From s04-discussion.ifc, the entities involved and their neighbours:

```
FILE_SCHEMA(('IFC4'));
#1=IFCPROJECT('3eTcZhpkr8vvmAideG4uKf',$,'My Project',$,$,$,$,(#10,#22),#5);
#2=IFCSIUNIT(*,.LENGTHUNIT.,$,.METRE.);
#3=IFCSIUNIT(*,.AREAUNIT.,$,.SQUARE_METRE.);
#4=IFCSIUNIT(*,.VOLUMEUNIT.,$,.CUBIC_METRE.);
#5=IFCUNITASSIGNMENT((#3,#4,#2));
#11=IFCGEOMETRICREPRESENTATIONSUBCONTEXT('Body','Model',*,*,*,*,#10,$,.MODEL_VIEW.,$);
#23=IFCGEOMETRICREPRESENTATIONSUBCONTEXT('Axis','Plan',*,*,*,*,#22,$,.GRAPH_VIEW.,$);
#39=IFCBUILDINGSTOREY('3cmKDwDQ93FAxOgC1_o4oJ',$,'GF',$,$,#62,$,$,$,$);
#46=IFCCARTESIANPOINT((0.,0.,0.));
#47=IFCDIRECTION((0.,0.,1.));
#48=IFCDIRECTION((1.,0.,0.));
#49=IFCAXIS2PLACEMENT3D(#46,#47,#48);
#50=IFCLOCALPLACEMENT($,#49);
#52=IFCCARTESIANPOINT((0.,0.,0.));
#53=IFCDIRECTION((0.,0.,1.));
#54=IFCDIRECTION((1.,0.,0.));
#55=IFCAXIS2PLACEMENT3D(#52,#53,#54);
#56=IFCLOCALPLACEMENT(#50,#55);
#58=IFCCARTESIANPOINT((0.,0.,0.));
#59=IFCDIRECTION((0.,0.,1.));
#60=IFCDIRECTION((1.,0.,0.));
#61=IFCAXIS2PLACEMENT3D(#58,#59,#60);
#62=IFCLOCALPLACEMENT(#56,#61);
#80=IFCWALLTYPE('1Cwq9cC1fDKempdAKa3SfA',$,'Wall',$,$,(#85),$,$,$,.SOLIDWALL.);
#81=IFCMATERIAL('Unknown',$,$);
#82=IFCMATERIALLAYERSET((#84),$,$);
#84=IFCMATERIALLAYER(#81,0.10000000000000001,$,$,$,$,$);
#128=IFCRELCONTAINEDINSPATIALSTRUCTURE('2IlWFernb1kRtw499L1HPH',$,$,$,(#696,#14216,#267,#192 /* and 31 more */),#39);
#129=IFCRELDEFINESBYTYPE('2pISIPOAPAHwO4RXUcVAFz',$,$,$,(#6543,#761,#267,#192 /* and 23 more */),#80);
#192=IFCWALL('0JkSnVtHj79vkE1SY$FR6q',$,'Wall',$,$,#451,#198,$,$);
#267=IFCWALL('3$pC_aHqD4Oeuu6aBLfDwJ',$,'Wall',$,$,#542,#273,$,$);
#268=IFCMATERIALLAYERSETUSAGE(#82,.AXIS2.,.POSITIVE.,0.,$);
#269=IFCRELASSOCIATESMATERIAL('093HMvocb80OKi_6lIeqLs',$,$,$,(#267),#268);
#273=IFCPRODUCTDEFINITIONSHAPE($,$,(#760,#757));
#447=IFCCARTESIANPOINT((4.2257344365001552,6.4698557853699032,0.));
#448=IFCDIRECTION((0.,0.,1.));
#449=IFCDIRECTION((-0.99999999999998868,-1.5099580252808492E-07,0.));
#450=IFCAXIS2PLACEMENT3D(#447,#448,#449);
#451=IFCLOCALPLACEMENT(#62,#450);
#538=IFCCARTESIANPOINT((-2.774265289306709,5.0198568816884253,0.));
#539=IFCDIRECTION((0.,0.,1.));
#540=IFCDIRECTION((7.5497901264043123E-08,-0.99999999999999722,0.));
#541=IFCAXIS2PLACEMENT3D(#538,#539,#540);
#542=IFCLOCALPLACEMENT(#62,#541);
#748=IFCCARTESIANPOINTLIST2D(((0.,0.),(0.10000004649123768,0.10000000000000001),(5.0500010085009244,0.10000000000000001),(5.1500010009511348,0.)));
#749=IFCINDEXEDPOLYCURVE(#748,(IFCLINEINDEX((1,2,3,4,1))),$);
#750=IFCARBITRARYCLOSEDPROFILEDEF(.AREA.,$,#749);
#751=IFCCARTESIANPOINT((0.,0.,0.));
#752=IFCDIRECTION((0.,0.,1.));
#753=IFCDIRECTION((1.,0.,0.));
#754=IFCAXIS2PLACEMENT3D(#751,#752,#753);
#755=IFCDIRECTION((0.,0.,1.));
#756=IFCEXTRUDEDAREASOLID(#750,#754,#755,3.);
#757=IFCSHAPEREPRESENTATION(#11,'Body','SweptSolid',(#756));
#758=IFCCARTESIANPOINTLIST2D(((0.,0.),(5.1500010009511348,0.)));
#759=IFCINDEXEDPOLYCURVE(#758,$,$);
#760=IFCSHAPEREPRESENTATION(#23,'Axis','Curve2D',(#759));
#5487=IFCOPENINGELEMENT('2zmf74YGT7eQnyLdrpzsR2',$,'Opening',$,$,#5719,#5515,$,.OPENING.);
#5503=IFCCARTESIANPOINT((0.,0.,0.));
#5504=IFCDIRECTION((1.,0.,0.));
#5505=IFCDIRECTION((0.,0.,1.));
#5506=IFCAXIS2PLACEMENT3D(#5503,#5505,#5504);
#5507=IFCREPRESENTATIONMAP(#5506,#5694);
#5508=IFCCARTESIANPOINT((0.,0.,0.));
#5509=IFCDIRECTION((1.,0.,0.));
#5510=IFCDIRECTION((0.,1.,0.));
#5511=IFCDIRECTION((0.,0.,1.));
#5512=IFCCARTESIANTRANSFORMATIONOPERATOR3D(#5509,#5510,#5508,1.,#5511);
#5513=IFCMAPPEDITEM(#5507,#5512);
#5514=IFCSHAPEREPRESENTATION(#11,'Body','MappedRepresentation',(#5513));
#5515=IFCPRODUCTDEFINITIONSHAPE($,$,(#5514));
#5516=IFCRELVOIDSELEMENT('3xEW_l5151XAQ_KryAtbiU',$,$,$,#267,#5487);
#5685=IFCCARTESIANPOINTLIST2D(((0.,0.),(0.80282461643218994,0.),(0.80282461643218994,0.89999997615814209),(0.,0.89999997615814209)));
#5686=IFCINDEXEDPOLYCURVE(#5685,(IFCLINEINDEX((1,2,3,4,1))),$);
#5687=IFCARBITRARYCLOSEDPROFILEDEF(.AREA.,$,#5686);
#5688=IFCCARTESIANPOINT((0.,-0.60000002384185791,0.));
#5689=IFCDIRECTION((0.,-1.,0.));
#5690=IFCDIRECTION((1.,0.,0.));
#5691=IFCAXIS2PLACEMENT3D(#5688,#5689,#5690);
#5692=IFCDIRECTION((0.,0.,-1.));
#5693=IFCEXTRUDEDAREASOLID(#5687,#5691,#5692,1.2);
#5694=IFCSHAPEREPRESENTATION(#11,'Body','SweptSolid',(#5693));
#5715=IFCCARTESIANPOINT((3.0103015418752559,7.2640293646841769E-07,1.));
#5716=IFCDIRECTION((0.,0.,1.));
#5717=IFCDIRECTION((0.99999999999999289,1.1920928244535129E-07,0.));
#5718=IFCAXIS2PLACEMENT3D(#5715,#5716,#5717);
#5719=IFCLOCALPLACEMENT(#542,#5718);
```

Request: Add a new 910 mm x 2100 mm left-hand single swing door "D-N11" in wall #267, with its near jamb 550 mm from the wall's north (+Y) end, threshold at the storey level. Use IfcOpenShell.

```python
import numpy as np
import ifcopenshell
import ifcopenshell.api.feature
import ifcopenshell.api.geometry
import ifcopenshell.api.root
import ifcopenshell.api.spatial
import ifcopenshell.geom
import ifcopenshell.util.element
import ifcopenshell.util.placement
import ifcopenshell.util.representation
import ifcopenshell.util.shape
import ifcopenshell.util.unit

model = ifcopenshell.open("s04-discussion.ifc")
unit_scale = ifcopenshell.util.unit.calculate_unit_scale(model)
settings = ifcopenshell.geom.settings()


def volume(element):
    """Net volume in cubic metres, openings subtracted."""
    shape = ifcopenshell.geom.create_shape(settings, element)
    return ifcopenshell.util.shape.get_volume(shape.geometry)


wall = model.by_id(267)
storey = ifcopenshell.util.element.get_container(wall, ifc_class="IfcBuildingStorey")
context = ifcopenshell.util.representation.get_context(model, "Model", "Body", "MODEL_VIEW")
before = volume(wall)

width, height, from_end, sill = 0.91, 2.1, 0.55, 0.0  # metres

# The wall runs along its own X axis, and the end named is its -X end.
wall_shape = ifcopenshell.geom.create_shape(settings, wall)
x, y, z = ifcopenshell.util.shape.get_vertices(wall_shape.geometry).T
start = x.min() + from_end
face, thickness = float(y.min()), float(y.max() - y.min())
wall_matrix = ifcopenshell.util.placement.get_local_placement(wall.ObjectPlacement)
level = ifcopenshell.util.placement.get_local_placement(storey.ObjectPlacement)[2, 3]


def in_wall(x, y):
    """Placement at x, y metres in the wall's axes, at sill height."""
    matrix = wall_matrix.copy()
    matrix[:, 3] = wall_matrix @ np.array([x / unit_scale, y / unit_scale, 0.0, 1.0])
    matrix[2, 3] = level + sill / unit_scale
    return matrix


# Opening: a box that overshoots both wall faces by 50 mm.
opening = ifcopenshell.api.root.create_entity(model, ifc_class="IfcOpeningElement", predefined_type="OPENING")
box = ifcopenshell.api.geometry.add_wall_representation(
    model, context=context, length=width, height=height, thickness=thickness + 0.1
)
ifcopenshell.api.geometry.assign_representation(model, product=opening, representation=box)
ifcopenshell.api.geometry.edit_object_placement(model, product=opening, matrix=in_wall(start, face - 0.05), is_si=False)
ifcopenshell.api.feature.add_feature(model, feature=opening, element=wall)

door = ifcopenshell.api.root.create_entity(model, ifc_class="IfcDoor", name="D-N11", predefined_type="DOOR")
door.OverallWidth, door.OverallHeight = width / unit_scale, height / unit_scale
door.OperationType = "SINGLE_SWING_LEFT"
body = ifcopenshell.api.geometry.add_door_representation(
    model,
    context=context,
    overall_width=door.OverallWidth,
    overall_height=door.OverallHeight,
    operation_type="SINGLE_SWING_LEFT",
    lining_properties={"LiningDepth": thickness / unit_scale, "ThresholdDepth": thickness / unit_scale},
)
ifcopenshell.api.geometry.assign_representation(model, product=door, representation=body)
ifcopenshell.api.spatial.assign_container(model, products=[door], relating_structure=storey)
ifcopenshell.api.feature.add_filling(model, opening=opening, element=door)

# The lining spans the wall, so the door starts at the wall face.
ifcopenshell.api.geometry.edit_object_placement(model, product=door, matrix=in_wall(start, face), is_si=False)

after = volume(wall)

print(f"wall volume {before:.3f} -> {after:.3f} m3")

model.write("s04-discussion_rev.ifc")
```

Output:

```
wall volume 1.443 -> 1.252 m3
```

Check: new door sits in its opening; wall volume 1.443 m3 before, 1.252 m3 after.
